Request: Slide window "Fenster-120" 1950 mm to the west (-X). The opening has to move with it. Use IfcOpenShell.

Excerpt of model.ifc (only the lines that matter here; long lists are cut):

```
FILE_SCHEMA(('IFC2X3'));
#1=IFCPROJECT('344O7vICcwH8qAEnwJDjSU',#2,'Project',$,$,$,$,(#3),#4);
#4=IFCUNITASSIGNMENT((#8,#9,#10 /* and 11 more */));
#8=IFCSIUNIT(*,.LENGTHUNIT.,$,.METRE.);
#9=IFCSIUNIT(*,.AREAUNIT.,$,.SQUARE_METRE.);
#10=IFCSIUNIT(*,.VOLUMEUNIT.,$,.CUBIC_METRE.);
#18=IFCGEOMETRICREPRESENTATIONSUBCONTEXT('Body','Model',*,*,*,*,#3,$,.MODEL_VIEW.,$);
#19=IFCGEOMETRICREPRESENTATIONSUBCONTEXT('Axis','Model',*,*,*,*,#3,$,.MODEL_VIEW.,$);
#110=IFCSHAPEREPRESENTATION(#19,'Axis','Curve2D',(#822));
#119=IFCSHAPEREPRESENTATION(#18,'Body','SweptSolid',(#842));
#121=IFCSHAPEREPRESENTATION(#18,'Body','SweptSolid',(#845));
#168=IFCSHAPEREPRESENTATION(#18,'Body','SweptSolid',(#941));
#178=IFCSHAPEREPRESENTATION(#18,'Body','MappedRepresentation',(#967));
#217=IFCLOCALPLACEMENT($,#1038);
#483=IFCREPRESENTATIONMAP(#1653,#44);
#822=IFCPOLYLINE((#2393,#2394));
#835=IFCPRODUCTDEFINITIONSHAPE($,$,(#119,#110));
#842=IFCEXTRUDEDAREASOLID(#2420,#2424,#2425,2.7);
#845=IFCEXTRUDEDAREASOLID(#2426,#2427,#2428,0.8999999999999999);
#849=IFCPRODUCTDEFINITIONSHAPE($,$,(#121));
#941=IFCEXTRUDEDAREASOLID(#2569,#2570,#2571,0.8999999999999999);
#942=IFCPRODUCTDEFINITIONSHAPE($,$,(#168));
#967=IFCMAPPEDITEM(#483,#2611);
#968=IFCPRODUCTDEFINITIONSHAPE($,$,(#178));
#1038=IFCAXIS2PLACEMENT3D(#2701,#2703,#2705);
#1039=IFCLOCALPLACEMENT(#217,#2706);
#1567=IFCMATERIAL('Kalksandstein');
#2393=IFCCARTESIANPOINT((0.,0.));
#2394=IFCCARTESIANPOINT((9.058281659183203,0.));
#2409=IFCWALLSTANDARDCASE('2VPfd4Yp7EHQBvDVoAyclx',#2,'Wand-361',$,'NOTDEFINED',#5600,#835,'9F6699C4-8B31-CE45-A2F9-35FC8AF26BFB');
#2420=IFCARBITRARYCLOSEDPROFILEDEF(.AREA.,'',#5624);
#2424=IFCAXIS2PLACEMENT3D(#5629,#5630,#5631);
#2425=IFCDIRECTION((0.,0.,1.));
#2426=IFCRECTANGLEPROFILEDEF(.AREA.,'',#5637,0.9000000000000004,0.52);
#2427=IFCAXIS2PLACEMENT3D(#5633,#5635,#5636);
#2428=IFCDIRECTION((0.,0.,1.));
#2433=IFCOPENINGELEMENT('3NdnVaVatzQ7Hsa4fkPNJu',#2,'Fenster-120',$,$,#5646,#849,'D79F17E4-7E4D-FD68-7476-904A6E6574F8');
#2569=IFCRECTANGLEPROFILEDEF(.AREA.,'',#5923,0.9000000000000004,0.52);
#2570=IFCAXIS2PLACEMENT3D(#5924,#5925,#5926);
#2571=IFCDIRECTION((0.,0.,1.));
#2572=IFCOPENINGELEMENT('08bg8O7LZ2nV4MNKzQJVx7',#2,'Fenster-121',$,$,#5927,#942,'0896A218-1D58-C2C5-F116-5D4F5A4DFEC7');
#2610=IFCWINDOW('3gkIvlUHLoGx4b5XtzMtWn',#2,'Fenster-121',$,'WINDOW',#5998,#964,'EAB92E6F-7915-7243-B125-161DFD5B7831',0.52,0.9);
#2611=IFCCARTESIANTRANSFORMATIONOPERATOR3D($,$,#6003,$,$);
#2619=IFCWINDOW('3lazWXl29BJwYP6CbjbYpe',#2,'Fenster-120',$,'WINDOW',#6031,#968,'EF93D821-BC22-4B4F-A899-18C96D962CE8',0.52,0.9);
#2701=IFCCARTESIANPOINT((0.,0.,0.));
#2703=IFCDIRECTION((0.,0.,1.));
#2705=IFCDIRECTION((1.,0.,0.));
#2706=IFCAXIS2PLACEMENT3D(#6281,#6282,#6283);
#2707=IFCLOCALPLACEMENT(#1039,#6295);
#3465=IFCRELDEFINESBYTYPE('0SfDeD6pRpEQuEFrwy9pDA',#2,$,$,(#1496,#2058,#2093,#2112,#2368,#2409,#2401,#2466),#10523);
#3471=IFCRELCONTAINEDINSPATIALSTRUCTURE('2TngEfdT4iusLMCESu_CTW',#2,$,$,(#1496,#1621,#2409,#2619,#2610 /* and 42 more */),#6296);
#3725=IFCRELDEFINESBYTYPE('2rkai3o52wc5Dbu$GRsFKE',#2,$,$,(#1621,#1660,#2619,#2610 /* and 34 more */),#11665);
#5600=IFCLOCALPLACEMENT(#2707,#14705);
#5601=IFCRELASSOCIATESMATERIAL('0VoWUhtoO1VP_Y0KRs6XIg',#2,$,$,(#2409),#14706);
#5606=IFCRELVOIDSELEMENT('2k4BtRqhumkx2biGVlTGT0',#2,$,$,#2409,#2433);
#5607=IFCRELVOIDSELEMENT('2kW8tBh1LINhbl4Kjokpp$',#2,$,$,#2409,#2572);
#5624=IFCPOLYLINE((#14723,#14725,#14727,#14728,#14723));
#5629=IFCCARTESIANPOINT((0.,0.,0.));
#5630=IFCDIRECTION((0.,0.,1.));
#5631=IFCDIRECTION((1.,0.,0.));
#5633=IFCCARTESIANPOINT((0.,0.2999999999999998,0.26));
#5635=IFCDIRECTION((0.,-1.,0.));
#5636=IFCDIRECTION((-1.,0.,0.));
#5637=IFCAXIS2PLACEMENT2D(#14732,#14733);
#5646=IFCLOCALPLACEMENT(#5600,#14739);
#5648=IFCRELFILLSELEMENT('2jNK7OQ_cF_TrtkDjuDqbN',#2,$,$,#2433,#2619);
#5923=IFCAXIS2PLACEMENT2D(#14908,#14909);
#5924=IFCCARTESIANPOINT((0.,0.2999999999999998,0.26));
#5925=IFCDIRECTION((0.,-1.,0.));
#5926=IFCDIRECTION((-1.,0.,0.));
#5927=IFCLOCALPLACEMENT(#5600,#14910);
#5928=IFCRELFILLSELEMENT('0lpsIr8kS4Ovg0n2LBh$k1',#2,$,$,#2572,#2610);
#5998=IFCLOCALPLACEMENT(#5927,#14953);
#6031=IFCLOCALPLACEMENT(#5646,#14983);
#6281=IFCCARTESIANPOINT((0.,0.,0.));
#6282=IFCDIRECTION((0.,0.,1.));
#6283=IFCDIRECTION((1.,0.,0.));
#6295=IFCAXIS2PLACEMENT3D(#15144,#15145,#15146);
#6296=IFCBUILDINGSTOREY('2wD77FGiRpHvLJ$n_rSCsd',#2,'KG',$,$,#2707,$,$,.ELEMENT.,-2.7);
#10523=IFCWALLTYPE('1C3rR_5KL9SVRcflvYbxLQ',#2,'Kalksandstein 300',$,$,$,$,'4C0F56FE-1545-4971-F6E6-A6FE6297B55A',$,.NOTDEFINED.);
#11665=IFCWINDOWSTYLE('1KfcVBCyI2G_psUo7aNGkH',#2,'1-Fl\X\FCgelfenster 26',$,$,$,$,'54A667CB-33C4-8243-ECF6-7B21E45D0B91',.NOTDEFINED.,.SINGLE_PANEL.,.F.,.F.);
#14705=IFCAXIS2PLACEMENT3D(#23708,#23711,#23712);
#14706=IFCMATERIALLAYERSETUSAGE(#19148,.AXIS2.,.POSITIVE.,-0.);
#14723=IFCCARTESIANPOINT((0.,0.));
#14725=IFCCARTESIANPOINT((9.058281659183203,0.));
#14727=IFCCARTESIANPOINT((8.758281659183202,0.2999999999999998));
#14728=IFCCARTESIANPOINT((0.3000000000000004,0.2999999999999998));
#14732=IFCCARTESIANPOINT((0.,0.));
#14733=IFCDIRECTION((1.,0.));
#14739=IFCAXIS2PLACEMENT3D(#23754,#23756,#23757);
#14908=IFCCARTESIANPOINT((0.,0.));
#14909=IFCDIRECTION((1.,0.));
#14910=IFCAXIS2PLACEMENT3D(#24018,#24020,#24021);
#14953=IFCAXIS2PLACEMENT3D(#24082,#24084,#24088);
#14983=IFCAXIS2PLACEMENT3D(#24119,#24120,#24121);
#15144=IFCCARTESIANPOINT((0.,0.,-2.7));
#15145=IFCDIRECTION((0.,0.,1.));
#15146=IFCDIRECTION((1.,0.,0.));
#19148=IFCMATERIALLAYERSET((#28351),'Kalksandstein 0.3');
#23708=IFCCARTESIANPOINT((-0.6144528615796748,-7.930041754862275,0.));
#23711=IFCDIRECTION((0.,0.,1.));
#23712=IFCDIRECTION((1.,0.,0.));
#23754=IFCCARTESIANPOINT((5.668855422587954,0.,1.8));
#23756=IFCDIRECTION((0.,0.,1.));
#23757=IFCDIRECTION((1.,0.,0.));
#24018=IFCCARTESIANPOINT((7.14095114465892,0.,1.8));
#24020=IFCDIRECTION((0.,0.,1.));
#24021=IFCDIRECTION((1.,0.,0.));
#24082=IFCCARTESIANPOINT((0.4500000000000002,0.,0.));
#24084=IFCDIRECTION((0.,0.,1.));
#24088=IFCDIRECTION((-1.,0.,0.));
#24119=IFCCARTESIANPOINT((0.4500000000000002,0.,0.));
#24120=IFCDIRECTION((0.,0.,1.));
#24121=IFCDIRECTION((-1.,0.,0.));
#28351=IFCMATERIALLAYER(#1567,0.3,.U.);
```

```python
import ifcopenshell
import ifcopenshell.api.geometry
import ifcopenshell.util.placement

model = ifcopenshell.open("model.ifc")

window = model.by_guid("3lazWXl29BJwYP6CbjbYpe")
opening = window.FillsVoids[0].RelatingOpeningElement
wall = opening.VoidsElements[0].RelatingBuildingElement

wall_matrix = ifcopenshell.util.placement.get_local_placement(wall.ObjectPlacement)
shift = wall_matrix[:3, 0] * -1.95
before = ifcopenshell.util.placement.get_local_placement(window.ObjectPlacement)[:3, 3].copy()

# The window is placed relative to its opening, so it follows when the opening moves.
matrix = ifcopenshell.util.placement.get_local_placement(opening.ObjectPlacement)
matrix[:3, 3] += shift
ifcopenshell.api.geometry.edit_object_placement(
    model, product=opening, matrix=matrix, is_si=False, should_transform_children=True
)

after = ifcopenshell.util.placement.get_local_placement(window.ObjectPlacement)[:3, 3]
print("window moved by", (after - before).round(3) + 0.0)

model.write("model_rev.ifc")
```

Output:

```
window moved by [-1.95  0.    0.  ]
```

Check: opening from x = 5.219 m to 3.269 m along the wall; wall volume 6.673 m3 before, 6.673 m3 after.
